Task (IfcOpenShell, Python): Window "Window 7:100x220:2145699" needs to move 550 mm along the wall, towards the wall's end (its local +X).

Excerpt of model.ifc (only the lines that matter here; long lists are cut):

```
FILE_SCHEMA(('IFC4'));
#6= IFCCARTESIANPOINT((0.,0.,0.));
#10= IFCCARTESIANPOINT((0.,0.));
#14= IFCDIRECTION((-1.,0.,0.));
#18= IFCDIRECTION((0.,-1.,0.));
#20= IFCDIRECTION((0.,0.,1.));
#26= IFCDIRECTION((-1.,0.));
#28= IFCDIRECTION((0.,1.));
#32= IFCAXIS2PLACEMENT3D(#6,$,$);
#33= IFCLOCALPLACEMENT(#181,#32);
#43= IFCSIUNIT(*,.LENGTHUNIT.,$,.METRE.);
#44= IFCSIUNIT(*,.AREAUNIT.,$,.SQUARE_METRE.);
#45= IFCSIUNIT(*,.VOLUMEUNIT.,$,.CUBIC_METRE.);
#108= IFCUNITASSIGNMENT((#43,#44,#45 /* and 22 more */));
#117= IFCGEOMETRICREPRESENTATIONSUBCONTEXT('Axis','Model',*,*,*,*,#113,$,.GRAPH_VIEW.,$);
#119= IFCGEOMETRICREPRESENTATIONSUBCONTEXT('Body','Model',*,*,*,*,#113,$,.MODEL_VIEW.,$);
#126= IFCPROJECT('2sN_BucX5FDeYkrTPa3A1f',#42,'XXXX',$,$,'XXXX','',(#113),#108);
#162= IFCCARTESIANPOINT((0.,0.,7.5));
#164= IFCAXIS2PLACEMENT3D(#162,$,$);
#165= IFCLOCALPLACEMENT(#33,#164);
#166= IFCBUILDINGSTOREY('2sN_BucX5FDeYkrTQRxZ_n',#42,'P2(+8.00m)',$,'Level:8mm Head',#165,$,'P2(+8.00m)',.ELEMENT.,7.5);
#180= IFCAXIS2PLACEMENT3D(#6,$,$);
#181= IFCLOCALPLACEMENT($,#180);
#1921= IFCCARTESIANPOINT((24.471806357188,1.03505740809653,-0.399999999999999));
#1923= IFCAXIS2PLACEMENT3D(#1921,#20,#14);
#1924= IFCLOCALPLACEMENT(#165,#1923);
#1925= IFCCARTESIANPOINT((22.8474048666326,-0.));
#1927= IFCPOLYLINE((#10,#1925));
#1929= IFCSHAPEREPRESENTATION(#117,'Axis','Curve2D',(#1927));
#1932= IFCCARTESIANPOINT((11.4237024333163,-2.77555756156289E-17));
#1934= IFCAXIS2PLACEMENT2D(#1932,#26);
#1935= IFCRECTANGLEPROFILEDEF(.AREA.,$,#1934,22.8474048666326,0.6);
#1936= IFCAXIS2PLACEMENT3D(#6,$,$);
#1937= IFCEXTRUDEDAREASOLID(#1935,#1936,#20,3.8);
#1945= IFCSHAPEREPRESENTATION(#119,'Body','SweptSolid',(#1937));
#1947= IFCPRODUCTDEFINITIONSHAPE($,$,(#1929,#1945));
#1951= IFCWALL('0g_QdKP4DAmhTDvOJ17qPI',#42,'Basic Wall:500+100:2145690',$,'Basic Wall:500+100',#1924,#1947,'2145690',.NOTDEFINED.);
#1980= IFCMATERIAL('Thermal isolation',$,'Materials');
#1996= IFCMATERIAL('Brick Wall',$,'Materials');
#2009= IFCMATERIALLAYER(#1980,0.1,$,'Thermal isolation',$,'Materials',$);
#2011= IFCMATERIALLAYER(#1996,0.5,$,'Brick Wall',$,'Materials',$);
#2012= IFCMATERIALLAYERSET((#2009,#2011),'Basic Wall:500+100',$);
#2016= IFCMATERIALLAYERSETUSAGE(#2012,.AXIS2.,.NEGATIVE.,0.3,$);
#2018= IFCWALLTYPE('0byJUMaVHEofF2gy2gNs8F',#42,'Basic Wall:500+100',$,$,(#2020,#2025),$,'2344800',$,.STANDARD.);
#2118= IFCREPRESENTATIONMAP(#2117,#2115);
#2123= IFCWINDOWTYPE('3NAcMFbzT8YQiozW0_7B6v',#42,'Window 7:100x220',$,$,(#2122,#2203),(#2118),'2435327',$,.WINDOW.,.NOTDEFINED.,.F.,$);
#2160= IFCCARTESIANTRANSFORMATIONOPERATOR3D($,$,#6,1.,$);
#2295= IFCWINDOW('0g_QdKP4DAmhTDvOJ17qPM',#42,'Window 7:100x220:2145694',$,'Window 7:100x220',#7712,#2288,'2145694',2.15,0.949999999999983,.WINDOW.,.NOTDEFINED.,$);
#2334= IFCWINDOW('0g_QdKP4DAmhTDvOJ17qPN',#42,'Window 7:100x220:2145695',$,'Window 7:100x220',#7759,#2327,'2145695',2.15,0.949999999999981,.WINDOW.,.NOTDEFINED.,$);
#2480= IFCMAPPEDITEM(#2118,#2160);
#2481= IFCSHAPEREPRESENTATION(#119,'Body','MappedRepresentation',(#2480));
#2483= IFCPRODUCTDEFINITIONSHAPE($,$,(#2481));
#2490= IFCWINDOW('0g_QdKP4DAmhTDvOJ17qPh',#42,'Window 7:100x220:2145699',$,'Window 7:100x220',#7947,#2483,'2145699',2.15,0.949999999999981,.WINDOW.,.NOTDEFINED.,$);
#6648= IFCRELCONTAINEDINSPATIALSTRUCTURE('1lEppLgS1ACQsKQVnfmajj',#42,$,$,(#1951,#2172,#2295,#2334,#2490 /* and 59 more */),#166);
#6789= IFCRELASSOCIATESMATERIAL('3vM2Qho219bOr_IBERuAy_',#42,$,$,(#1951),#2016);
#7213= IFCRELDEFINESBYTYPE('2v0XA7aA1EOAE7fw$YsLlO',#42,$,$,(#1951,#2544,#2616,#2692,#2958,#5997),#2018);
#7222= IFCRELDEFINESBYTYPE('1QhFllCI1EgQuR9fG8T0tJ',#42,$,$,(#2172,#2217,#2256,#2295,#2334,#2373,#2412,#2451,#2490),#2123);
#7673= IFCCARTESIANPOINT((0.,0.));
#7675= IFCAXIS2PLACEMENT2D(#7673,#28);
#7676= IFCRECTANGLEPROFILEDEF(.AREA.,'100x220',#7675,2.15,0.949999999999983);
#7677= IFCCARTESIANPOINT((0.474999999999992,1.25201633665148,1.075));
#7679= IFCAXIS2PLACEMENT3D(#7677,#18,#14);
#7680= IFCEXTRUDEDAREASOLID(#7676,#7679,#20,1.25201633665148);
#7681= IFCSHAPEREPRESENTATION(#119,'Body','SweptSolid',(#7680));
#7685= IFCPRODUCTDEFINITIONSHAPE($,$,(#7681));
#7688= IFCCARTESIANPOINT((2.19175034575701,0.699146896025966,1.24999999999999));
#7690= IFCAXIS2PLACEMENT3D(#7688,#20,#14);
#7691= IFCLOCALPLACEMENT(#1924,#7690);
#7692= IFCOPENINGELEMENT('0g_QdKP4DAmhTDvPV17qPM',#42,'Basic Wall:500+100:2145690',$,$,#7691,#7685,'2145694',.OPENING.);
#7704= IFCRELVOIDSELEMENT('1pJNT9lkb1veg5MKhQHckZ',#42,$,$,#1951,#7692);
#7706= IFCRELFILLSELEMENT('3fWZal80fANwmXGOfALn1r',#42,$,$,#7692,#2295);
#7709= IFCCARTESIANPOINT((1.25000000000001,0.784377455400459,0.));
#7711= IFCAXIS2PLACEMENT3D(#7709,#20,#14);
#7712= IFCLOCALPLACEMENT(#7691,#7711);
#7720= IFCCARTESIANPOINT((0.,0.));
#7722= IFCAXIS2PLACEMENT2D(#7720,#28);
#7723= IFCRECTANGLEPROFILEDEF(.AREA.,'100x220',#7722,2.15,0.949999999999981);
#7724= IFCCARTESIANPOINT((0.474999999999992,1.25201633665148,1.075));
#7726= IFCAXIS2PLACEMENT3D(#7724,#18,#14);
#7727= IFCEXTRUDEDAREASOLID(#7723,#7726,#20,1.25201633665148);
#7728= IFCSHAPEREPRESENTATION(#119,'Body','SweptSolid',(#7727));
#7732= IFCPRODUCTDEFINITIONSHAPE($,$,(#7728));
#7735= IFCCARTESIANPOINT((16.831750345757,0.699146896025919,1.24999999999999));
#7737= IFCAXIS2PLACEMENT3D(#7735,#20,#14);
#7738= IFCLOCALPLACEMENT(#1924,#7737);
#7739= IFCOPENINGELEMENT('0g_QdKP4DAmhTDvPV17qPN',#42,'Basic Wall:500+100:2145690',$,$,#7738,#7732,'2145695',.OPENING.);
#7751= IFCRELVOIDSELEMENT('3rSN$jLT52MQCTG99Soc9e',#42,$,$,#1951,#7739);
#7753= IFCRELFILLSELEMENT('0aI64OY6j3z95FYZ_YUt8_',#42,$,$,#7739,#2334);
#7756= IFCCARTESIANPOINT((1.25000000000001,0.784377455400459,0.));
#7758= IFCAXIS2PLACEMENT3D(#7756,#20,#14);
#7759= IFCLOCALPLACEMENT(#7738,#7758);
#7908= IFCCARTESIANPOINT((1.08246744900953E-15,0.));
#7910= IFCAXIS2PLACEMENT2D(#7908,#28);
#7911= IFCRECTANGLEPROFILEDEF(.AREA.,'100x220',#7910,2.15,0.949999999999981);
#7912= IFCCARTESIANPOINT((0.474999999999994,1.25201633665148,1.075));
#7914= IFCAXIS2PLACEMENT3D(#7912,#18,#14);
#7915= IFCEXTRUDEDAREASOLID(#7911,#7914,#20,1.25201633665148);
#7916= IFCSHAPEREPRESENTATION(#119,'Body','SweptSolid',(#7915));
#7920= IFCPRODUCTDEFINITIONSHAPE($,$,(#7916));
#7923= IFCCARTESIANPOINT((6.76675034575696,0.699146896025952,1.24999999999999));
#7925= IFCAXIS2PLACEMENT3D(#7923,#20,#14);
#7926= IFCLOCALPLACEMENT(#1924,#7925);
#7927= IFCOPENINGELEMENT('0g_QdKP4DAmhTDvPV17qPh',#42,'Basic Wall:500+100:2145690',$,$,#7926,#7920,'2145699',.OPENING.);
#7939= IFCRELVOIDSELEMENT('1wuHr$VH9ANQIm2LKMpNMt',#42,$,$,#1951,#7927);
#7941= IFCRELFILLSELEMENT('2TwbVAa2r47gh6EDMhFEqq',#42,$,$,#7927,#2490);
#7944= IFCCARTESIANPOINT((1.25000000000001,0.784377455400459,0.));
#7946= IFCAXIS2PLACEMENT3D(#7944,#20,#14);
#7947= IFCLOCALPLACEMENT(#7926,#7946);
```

```python
import ifcopenshell
import ifcopenshell.api.geometry
import ifcopenshell.util.placement
import ifcopenshell.util.unit

model = ifcopenshell.open("model.ifc")
unit_scale = ifcopenshell.util.unit.calculate_unit_scale(model)

window = model.by_guid("0g_QdKP4DAmhTDvOJ17qPh")
opening = window.FillsVoids[0].RelatingOpeningElement
wall = opening.VoidsElements[0].RelatingBuildingElement

wall_matrix = ifcopenshell.util.placement.get_local_placement(wall.ObjectPlacement)
shift = wall_matrix[:3, 0] * 0.55 / unit_scale
before = ifcopenshell.util.placement.get_local_placement(window.ObjectPlacement)[:3, 3].copy()

# The window is placed relative to its opening, so it follows when the opening moves.
matrix = ifcopenshell.util.placement.get_local_placement(opening.ObjectPlacement)
matrix[:3, 3] += shift
ifcopenshell.api.geometry.edit_object_placement(
    model, product=opening, matrix=matrix, is_si=False, should_transform_children=True
)

after = ifcopenshell.util.placement.get_local_placement(window.ObjectPlacement)[:3, 3]
print("window moved by", (after - before).round(3) + 0.0)

model.write("model_updated.ifc")
```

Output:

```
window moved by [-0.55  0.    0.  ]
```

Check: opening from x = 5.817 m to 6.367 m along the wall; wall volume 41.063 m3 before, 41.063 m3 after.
